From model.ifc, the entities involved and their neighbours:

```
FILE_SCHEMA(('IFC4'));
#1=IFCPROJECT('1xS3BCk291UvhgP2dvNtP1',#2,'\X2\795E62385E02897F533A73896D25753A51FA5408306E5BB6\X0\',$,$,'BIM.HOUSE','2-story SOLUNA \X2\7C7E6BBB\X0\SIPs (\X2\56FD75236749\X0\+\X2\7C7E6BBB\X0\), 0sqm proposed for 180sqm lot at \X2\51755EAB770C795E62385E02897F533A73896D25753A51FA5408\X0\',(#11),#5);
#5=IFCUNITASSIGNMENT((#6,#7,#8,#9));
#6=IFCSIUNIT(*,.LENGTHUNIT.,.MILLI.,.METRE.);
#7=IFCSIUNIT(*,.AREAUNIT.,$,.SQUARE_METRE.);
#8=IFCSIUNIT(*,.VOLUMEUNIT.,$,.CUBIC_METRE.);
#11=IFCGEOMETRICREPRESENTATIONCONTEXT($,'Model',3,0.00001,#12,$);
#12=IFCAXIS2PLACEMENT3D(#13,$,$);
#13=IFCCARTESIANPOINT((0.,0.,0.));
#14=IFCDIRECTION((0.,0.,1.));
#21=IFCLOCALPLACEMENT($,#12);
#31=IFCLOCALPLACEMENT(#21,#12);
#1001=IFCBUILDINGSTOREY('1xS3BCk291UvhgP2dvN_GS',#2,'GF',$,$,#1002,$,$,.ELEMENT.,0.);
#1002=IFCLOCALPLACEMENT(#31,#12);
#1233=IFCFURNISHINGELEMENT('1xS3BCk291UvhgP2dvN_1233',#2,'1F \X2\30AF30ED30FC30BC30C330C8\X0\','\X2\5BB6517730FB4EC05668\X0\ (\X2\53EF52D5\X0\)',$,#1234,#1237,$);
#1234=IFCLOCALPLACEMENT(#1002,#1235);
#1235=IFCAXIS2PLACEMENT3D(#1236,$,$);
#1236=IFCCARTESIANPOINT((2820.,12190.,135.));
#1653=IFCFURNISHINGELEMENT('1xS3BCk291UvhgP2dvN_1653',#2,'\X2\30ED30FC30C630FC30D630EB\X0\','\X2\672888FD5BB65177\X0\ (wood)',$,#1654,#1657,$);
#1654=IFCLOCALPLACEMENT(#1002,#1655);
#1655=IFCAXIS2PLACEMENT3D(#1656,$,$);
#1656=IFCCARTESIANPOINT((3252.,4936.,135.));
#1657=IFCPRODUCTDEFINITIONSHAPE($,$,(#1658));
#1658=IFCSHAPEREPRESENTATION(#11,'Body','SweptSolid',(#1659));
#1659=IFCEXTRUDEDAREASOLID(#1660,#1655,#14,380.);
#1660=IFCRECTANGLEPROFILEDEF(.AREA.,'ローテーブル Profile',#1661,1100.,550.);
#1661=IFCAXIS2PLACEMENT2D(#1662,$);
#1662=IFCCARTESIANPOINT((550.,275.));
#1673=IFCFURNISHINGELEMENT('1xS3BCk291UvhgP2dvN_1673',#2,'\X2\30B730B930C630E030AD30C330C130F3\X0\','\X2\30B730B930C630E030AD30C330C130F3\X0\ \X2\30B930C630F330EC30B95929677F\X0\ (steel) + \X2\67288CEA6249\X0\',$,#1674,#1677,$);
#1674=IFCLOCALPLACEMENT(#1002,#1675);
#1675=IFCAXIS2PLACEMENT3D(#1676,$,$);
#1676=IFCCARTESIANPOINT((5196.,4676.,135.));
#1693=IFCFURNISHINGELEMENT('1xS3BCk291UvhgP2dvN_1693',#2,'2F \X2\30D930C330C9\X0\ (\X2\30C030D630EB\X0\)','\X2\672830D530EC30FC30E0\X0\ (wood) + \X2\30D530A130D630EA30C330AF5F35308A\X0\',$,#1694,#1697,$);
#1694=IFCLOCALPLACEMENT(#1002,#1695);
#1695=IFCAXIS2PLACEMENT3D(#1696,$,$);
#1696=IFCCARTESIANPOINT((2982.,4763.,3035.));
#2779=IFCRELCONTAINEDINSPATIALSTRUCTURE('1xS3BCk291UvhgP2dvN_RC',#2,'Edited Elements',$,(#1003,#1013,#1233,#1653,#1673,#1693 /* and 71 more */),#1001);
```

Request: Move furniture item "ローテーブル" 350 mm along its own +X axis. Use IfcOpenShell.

```python
import ifcopenshell
import ifcopenshell.api.geometry
import ifcopenshell.util.placement
import ifcopenshell.util.unit

model = ifcopenshell.open("model.ifc")
unit_scale = ifcopenshell.util.unit.calculate_unit_scale(model)

item = model.by_id(1653)
matrix = ifcopenshell.util.placement.get_local_placement(item.ObjectPlacement)
matrix[:3, 3] += matrix[:3, 0] * 0.35 / unit_scale
ifcopenshell.api.geometry.edit_object_placement(model, product=item, matrix=matrix, is_si=False)

print(ifcopenshell.util.placement.get_local_placement(item.ObjectPlacement).round(3) + 0.0)

model.write("model-out.ifc")
```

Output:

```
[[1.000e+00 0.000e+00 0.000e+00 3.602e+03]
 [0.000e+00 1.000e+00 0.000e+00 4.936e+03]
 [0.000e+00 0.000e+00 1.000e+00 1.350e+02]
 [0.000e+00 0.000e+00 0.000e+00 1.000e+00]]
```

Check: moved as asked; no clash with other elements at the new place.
